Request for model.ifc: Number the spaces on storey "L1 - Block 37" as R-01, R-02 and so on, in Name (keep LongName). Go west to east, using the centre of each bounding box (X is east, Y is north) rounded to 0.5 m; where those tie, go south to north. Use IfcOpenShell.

First a look at what the model holds.

```python
import ifcopenshell
import ifcopenshell.util.element
import ifcopenshell.util.placement

model = ifcopenshell.open("model.ifc")
print(model.schema)
storey = next(s for s in model.by_type("IfcBuildingStorey") if s.Name == "L1 - Block 37")
spaces = [e for e in ifcopenshell.util.element.get_decomposition(storey) if e.is_a("IfcSpace")]
for e in sorted(spaces, key=lambda e: e.id()):
    origin = ifcopenshell.util.placement.get_local_placement(e.ObjectPlacement)[:3, 3]
    print(e.id(), e.Name, e.LongName, origin.round(2) + 0.0, sep=" | ")
```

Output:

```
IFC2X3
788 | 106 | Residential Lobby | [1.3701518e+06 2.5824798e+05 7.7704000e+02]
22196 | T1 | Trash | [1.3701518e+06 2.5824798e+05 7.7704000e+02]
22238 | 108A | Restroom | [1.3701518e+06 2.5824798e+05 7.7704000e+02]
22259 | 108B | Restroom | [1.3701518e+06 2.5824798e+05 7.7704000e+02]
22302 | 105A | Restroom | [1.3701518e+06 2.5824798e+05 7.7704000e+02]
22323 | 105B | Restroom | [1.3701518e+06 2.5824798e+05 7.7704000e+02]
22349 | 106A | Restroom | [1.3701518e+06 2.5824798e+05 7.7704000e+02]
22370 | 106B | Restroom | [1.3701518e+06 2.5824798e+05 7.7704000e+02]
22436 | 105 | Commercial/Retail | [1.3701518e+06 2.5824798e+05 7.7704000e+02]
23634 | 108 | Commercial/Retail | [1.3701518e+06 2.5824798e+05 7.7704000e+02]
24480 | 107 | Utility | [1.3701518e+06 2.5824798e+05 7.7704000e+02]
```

```python
import ifcopenshell
import ifcopenshell.geom
import ifcopenshell.util.element
import ifcopenshell.util.shape

model = ifcopenshell.open("model.ifc")
settings = ifcopenshell.geom.settings()
settings.set("use-world-coords", True)


def centre(element):
    shape = ifcopenshell.geom.create_shape(settings, element)
    return ifcopenshell.util.shape.get_bbox_centroid(shape.geometry)


storey = next(s for s in model.by_type("IfcBuildingStorey") if s.Name == "L1 - Block 37")
spaces = [e for e in ifcopenshell.util.element.get_decomposition(storey) if e.is_a("IfcSpace")]

# Insertion points can sit at a corner or the storey origin, so sort by the geometry (in metres).
centres = {e: centre(e) for e in spaces}
spaces.sort(key=lambda e: (round(centres[e][0] / 0.5), centres[e][1]))

for i, e in enumerate(spaces, start=1):
    number = f"R-{i:02d}"
    e.Name = number
    print(e.id(), number)

model.write("model_edited.ifc")
```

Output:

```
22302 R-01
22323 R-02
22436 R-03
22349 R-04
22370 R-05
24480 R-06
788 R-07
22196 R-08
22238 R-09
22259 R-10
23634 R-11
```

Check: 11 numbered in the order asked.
